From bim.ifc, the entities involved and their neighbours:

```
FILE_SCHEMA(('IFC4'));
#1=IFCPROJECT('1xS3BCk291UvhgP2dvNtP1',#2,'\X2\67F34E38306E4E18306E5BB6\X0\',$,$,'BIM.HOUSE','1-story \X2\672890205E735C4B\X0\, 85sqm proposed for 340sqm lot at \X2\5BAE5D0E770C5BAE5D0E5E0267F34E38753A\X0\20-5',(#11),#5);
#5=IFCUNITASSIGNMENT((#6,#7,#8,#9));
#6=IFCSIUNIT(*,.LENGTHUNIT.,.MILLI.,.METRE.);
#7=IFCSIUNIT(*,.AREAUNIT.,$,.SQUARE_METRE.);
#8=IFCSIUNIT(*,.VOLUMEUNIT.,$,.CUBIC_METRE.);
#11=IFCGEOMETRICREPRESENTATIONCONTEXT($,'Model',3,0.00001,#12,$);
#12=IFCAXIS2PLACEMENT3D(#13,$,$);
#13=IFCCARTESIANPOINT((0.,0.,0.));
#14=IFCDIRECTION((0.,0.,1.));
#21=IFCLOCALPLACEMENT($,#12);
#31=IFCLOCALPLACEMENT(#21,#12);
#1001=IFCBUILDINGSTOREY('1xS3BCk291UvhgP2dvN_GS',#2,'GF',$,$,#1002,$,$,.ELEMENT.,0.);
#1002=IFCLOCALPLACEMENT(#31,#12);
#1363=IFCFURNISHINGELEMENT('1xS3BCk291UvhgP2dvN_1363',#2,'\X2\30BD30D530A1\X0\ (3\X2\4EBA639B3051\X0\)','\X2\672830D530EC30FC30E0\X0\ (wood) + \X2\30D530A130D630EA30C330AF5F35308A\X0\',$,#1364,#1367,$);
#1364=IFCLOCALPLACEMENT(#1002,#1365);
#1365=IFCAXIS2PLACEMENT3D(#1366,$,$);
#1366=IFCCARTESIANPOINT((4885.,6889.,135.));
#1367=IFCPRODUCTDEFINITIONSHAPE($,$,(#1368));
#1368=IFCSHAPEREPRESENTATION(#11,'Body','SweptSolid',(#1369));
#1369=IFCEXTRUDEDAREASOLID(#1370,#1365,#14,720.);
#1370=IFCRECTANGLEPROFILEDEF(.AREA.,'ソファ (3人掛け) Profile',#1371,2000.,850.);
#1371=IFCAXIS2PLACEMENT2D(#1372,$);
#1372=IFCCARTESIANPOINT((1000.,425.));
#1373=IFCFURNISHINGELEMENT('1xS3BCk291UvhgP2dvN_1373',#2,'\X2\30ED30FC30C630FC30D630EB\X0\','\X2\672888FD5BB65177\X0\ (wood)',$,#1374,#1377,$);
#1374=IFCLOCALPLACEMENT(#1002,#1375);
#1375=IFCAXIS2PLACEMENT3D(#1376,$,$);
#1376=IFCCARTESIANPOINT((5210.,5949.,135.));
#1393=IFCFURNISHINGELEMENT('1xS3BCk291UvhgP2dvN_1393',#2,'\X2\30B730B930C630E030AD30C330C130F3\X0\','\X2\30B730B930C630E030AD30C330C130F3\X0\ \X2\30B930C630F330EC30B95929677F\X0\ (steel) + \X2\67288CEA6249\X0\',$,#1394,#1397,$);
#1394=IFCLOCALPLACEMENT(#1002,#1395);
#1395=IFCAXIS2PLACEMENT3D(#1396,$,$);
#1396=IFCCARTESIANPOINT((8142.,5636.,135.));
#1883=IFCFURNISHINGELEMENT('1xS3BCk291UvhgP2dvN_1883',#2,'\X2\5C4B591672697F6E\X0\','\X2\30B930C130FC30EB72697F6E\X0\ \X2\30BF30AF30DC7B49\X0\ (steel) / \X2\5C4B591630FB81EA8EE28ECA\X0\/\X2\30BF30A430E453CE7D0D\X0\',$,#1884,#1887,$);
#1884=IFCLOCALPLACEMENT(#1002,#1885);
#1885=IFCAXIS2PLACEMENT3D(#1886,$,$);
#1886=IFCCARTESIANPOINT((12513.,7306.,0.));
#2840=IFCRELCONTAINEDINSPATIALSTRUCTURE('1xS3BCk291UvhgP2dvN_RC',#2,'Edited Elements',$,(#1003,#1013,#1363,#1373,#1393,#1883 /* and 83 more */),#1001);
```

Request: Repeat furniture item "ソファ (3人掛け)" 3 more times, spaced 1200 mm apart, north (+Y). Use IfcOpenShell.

```python
import numpy as np
import ifcopenshell
import ifcopenshell.api.geometry
import ifcopenshell.api.root
import ifcopenshell.util.element
import ifcopenshell.util.placement
import ifcopenshell.util.unit

model = ifcopenshell.open("bim.ifc")
unit_scale = ifcopenshell.util.unit.calculate_unit_scale(model)


def reuse_history(source, copy):
    """copy_class also copies each property set's owner history, people and application; keep the originals."""
    for rel in copy.IsDefinedBy:
        if rel.is_a("IfcRelDefinesByProperties") and (history := rel.RelatingPropertyDefinition.OwnerHistory):
            rel.RelatingPropertyDefinition.OwnerHistory = source.OwnerHistory
            ifcopenshell.util.element.remove_deep2(model, history)


source = model.by_guid("1xS3BCk291UvhgP2dvN_1363")
base = ifcopenshell.util.placement.get_local_placement(source.ObjectPlacement)
step = np.array([0.0, 1.0, 0.0]) * 1.2 / unit_scale

for i in range(1, 4):
    copy = ifcopenshell.api.root.copy_class(model, product=source)
    copy.Representation = ifcopenshell.util.element.copy_deep(
        model, source.Representation, exclude=["IfcGeometricRepresentationContext", "IfcRepresentationMap"]
    )
    reuse_history(source, copy)
    matrix = base.copy()
    matrix[:3, 3] += i * step
    print("added at", matrix[:3, 3].round(3) + 0.0)
    ifcopenshell.api.geometry.edit_object_placement(model, product=copy, matrix=matrix, is_si=False)

model.write("bim_edited.ifc")
```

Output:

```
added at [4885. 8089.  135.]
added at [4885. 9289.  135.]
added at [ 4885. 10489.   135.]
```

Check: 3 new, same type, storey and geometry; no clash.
